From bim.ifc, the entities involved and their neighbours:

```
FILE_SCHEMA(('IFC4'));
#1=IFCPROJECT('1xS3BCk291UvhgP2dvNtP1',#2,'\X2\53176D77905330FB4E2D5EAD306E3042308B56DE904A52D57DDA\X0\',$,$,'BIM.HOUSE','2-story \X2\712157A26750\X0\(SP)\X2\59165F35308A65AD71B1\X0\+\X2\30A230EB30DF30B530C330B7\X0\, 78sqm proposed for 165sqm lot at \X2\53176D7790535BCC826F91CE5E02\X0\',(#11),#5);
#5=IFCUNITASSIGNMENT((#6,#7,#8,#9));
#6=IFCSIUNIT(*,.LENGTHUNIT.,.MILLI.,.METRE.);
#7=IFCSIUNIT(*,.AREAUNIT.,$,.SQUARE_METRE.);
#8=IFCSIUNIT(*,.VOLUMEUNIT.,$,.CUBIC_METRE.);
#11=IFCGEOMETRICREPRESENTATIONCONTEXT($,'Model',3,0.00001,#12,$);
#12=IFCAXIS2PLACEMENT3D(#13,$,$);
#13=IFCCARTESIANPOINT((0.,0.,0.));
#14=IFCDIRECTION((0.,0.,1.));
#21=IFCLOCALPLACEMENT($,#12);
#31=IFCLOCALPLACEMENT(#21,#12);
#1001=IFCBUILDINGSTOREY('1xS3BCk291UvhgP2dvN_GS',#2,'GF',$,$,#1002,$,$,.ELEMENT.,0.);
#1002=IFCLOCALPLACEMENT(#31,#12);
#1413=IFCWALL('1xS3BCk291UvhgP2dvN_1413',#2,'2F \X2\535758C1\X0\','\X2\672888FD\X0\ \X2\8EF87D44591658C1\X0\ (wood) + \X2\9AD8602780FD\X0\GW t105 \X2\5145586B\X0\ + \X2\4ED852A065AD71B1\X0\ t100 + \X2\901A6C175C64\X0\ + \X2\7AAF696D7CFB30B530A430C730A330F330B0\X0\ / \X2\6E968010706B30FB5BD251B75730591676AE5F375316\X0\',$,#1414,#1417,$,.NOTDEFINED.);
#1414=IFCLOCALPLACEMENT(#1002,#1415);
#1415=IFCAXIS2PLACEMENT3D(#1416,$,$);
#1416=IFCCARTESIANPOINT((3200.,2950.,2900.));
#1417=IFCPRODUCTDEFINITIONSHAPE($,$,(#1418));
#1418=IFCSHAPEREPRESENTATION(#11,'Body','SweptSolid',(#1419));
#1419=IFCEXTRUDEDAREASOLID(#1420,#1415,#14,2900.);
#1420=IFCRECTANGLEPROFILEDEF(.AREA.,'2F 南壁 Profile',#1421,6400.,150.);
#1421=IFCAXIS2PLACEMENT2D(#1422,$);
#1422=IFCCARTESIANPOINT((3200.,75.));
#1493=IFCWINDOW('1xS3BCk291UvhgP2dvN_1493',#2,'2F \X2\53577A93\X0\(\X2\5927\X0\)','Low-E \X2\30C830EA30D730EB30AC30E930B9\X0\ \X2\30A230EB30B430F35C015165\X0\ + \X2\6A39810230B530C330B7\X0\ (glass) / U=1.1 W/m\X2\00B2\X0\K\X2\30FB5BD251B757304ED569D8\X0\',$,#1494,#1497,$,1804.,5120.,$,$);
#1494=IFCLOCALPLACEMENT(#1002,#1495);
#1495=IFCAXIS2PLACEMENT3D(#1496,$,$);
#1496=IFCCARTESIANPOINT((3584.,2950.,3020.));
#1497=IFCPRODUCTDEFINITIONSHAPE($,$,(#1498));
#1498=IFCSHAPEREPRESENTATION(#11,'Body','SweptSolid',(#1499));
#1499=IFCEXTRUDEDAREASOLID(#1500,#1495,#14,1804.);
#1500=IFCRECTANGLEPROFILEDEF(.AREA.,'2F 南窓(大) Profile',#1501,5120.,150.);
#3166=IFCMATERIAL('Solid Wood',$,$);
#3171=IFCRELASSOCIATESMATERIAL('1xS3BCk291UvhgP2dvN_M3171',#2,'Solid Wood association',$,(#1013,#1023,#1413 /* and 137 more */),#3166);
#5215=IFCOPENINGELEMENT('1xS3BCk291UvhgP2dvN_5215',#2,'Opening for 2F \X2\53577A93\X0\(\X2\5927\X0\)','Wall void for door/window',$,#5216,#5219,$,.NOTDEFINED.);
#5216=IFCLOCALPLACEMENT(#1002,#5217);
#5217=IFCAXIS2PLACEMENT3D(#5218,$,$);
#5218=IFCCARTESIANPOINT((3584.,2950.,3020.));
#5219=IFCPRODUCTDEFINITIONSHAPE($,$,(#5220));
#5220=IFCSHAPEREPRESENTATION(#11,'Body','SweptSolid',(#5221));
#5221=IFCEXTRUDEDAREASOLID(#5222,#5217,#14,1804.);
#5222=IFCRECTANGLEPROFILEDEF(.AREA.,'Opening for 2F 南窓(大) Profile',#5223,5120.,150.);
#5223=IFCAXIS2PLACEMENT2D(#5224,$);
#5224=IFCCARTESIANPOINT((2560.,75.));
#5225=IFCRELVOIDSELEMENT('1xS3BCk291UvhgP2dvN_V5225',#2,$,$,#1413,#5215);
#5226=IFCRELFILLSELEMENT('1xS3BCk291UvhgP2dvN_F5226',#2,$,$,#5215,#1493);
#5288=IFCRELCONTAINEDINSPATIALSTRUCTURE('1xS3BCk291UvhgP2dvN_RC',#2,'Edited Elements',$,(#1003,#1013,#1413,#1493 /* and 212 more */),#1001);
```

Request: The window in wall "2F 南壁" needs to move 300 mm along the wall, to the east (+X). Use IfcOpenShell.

```python
import ifcopenshell
import ifcopenshell.api.geometry
import ifcopenshell.util.placement

model = ifcopenshell.open("bim.ifc")

window = model.by_guid("1xS3BCk291UvhgP2dvN_1493")
opening = window.FillsVoids[0].RelatingOpeningElement
wall = opening.VoidsElements[0].RelatingBuildingElement

wall_matrix = ifcopenshell.util.placement.get_local_placement(wall.ObjectPlacement)
shift = wall_matrix[:3, 0] * 300.0
before = ifcopenshell.util.placement.get_local_placement(window.ObjectPlacement)[:3, 3].copy()

# The window is not placed relative to its opening, so move both.
for product in (opening, window):
    matrix = ifcopenshell.util.placement.get_local_placement(product.ObjectPlacement)
    matrix[:3, 3] += shift
    ifcopenshell.api.geometry.edit_object_placement(model, product=product, matrix=matrix, is_si=False)

after = ifcopenshell.util.placement.get_local_placement(window.ObjectPlacement)[:3, 3]
print("window moved by", (after - before).round(3) + 0.0)

model.write("bim_rev.ifc")
```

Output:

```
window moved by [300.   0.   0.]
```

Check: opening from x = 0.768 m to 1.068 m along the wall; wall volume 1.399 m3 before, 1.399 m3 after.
